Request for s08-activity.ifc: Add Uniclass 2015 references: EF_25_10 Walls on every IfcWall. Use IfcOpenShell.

First a look at what the model holds.

```python
import ifcopenshell

model = ifcopenshell.open("s08-activity.ifc")
print(model.schema)
print("classifications:", [c.Name for c in model.by_type("IfcClassification")])
for ifc_class in ("IfcDoor", "IfcRoof", "IfcStair", "IfcWall", "IfcWindow"):
    print(ifc_class, len(model.by_type(ifc_class)))
```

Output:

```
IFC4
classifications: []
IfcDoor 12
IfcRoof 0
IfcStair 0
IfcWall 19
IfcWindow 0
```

```python
import ifcopenshell
import ifcopenshell.api.classification

model = ifcopenshell.open("s08-activity.ifc")

system = ifcopenshell.api.classification.add_classification(model, classification="Uniclass 2015")

codes = {
    "IfcWall": ("EF_25_10", "Walls"),
}
for ifc_class, (code, name) in codes.items():
    products = model.by_type(ifc_class)
    ifcopenshell.api.classification.add_reference(
        model, products=products, classification=system, identification=code, name=name
    )
    print(code, len(products))

model.write("s08-activity_v2.ifc")
```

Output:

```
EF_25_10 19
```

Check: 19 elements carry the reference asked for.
